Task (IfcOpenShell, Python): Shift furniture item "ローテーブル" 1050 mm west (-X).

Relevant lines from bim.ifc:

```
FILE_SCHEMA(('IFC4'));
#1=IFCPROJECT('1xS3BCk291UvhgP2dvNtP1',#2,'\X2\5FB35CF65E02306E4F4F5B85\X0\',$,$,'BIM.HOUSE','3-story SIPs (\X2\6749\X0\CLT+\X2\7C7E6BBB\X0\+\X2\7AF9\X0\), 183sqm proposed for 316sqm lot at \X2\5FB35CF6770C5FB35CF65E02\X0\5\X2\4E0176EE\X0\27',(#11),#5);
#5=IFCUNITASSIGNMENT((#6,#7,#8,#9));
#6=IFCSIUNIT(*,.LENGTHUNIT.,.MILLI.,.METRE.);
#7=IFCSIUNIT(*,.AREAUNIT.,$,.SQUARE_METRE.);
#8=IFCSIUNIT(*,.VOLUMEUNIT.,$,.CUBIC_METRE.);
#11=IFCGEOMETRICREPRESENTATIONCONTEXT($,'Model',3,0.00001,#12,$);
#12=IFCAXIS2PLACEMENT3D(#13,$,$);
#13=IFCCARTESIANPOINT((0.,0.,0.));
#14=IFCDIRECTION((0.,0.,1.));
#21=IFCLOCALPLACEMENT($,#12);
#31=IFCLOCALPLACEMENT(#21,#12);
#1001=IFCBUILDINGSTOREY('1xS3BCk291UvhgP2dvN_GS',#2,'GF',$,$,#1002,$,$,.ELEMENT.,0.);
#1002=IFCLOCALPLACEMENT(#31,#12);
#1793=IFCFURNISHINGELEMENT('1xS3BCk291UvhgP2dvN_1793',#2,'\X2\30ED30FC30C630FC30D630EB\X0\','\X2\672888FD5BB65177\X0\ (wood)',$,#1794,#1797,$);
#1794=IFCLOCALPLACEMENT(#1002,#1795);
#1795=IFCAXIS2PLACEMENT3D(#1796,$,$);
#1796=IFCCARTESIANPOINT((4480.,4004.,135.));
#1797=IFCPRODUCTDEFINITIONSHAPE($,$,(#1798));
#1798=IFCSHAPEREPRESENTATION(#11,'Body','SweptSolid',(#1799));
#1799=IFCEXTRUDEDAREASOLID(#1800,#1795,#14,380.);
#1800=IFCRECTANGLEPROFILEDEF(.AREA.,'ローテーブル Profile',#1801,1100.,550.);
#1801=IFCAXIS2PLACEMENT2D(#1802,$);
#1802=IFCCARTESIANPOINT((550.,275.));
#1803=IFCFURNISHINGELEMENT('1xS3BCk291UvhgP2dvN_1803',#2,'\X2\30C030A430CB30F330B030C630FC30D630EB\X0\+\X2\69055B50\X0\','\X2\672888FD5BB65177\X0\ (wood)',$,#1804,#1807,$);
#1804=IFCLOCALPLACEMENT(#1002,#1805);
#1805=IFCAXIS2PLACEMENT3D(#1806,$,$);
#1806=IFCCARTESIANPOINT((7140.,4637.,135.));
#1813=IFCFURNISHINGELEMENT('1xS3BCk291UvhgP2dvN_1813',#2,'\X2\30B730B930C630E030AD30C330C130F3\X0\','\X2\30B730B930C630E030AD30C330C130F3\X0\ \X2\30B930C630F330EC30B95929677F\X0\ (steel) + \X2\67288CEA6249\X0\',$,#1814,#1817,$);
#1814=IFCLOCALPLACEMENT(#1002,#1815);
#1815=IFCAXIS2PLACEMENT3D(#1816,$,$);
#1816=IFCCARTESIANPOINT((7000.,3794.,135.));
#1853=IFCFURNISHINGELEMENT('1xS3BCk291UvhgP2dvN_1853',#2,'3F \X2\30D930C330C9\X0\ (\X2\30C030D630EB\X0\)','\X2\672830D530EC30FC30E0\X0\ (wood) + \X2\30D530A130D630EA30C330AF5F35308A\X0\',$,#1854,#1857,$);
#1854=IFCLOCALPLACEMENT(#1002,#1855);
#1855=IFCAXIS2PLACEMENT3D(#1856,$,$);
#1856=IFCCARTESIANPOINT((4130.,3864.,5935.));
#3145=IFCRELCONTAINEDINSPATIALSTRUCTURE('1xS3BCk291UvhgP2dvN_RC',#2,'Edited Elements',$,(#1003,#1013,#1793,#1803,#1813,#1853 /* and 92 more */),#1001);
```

```python
import ifcopenshell
import ifcopenshell.api.geometry
import ifcopenshell.util.placement

model = ifcopenshell.open("bim.ifc")

item = model.by_guid("1xS3BCk291UvhgP2dvN_1793")
matrix = ifcopenshell.util.placement.get_local_placement(item.ObjectPlacement)
matrix[0, 3] -= 1050.0
ifcopenshell.api.geometry.edit_object_placement(model, product=item, matrix=matrix, is_si=False)

print(ifcopenshell.util.placement.get_local_placement(item.ObjectPlacement).round(3) + 0.0)

model.write("bim_updated.ifc")
```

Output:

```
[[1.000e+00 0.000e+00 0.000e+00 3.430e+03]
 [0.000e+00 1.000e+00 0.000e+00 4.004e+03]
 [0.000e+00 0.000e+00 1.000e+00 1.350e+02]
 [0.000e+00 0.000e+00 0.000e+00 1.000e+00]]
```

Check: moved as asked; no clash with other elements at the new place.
